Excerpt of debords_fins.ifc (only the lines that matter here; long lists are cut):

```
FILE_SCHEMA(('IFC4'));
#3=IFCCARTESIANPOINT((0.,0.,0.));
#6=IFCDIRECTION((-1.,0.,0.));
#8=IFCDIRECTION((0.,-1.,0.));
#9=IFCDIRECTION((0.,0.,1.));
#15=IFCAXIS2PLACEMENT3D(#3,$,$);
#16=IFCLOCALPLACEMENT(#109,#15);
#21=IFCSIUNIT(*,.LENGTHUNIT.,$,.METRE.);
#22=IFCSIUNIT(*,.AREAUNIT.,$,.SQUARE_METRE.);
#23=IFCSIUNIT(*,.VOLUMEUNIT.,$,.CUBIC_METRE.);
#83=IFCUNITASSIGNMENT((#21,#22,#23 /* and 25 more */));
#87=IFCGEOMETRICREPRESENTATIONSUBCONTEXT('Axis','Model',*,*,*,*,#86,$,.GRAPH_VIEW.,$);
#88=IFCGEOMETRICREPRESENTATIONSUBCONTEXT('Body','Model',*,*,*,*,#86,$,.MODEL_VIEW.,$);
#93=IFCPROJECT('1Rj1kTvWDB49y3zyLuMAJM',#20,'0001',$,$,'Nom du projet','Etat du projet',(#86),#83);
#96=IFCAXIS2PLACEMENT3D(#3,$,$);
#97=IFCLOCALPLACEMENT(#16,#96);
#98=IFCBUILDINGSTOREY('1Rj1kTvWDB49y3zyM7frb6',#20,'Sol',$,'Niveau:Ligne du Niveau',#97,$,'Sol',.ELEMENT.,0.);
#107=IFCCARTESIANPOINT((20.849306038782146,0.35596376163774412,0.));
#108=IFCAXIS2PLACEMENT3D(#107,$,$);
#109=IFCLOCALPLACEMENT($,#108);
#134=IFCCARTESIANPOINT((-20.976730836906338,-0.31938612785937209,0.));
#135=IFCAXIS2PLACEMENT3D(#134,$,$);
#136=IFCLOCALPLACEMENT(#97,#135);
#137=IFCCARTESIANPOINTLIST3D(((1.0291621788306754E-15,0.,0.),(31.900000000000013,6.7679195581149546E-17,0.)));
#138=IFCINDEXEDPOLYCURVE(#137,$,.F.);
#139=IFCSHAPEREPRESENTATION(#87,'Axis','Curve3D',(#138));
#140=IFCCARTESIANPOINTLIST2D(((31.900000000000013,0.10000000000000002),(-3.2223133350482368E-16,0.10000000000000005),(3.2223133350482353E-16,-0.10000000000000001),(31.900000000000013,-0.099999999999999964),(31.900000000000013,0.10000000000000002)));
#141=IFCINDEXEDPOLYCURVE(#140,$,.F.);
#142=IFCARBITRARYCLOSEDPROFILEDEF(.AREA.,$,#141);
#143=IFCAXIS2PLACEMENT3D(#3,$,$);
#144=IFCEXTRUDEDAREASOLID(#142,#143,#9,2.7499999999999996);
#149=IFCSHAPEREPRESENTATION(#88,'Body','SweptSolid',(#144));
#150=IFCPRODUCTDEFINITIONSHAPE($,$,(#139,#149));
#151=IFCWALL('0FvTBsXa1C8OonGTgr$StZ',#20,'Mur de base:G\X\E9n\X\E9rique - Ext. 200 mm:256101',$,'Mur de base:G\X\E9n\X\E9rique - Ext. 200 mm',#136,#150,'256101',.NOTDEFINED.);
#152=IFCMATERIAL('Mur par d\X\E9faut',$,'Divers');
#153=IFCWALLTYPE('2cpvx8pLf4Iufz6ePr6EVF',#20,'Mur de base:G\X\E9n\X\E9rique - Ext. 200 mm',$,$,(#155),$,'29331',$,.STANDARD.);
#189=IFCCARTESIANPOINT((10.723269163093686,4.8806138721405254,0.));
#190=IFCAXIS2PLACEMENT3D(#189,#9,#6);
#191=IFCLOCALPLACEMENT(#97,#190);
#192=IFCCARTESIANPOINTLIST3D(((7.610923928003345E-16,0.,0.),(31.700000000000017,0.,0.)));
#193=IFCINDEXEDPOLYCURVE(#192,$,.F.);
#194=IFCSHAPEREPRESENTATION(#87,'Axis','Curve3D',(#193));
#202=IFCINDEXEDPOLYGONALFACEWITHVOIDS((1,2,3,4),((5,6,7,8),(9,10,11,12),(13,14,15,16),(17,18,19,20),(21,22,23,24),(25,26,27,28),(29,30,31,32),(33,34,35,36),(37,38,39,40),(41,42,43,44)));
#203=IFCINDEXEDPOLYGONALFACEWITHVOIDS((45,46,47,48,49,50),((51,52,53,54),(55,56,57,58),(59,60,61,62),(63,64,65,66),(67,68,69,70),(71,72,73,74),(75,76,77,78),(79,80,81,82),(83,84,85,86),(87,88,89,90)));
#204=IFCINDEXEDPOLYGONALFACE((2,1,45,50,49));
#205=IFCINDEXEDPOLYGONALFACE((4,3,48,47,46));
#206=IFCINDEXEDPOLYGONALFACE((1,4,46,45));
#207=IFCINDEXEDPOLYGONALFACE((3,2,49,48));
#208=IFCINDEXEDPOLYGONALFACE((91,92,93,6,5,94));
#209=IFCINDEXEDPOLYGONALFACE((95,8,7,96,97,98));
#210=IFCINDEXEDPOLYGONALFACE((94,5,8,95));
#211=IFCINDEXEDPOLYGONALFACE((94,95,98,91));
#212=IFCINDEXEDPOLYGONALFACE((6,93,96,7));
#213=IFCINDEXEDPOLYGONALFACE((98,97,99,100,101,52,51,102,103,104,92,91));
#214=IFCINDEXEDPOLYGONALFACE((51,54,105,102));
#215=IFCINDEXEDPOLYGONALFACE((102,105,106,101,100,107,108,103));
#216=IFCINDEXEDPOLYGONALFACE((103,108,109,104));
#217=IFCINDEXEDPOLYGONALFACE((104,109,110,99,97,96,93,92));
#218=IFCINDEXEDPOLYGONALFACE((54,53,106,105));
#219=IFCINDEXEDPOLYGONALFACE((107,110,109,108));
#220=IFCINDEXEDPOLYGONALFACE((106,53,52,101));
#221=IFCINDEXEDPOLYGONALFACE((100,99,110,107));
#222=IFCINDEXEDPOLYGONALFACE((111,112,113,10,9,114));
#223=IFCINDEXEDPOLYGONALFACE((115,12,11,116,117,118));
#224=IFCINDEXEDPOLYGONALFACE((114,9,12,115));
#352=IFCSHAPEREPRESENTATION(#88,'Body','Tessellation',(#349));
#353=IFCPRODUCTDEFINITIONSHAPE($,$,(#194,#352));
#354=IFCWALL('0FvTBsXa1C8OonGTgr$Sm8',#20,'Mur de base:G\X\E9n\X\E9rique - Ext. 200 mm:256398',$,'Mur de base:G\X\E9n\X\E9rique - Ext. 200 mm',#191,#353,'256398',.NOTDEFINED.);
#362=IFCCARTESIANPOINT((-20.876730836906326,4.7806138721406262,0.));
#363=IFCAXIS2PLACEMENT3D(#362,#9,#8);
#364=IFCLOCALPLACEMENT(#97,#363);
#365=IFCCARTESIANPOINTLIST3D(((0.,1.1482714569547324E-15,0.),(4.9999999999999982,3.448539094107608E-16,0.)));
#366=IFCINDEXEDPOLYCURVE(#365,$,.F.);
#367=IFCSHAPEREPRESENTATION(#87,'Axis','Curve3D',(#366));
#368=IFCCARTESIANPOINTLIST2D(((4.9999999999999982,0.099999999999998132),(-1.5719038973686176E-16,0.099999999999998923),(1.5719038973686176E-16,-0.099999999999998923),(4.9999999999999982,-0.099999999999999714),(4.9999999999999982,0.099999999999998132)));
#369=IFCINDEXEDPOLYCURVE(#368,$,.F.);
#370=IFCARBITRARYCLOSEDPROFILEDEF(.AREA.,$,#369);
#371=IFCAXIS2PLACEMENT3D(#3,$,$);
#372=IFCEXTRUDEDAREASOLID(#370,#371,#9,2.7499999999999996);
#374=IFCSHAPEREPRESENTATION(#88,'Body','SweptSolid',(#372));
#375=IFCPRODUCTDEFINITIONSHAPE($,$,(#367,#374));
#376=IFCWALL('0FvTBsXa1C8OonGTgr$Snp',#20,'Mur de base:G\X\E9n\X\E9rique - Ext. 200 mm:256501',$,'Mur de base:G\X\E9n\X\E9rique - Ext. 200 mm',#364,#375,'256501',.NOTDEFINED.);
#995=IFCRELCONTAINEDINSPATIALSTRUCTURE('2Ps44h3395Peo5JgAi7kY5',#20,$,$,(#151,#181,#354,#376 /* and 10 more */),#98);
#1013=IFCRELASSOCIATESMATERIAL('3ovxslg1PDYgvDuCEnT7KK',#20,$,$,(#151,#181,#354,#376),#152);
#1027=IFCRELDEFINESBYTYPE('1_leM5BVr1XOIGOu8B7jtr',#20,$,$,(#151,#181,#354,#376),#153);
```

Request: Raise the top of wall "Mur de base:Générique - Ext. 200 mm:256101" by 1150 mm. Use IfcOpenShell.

```python
import ifcopenshell
import ifcopenshell.geom
import ifcopenshell.util.representation
import ifcopenshell.util.shape

model = ifcopenshell.open("debords_fins.ifc")
settings = ifcopenshell.geom.settings()


def volume(element):
    """Net volume in cubic metres, openings subtracted."""
    shape = ifcopenshell.geom.create_shape(settings, element)
    return ifcopenshell.util.shape.get_volume(shape.geometry)


wall = model.by_guid("0FvTBsXa1C8OonGTgr$StZ")
before = volume(wall)

body = ifcopenshell.util.representation.get_representation(wall, "Model", "Body")
solid = body.Items[0]
old_height = solid.Depth
solid.Depth += 1.15
after = volume(wall)

print(f"height {old_height:g} -> {solid.Depth:g}, volume {before:.3f} -> {after:.3f} m3")

model.write("debords_fins_rev.ifc")
```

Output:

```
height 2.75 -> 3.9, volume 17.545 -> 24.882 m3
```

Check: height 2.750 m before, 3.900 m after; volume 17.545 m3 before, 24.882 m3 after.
